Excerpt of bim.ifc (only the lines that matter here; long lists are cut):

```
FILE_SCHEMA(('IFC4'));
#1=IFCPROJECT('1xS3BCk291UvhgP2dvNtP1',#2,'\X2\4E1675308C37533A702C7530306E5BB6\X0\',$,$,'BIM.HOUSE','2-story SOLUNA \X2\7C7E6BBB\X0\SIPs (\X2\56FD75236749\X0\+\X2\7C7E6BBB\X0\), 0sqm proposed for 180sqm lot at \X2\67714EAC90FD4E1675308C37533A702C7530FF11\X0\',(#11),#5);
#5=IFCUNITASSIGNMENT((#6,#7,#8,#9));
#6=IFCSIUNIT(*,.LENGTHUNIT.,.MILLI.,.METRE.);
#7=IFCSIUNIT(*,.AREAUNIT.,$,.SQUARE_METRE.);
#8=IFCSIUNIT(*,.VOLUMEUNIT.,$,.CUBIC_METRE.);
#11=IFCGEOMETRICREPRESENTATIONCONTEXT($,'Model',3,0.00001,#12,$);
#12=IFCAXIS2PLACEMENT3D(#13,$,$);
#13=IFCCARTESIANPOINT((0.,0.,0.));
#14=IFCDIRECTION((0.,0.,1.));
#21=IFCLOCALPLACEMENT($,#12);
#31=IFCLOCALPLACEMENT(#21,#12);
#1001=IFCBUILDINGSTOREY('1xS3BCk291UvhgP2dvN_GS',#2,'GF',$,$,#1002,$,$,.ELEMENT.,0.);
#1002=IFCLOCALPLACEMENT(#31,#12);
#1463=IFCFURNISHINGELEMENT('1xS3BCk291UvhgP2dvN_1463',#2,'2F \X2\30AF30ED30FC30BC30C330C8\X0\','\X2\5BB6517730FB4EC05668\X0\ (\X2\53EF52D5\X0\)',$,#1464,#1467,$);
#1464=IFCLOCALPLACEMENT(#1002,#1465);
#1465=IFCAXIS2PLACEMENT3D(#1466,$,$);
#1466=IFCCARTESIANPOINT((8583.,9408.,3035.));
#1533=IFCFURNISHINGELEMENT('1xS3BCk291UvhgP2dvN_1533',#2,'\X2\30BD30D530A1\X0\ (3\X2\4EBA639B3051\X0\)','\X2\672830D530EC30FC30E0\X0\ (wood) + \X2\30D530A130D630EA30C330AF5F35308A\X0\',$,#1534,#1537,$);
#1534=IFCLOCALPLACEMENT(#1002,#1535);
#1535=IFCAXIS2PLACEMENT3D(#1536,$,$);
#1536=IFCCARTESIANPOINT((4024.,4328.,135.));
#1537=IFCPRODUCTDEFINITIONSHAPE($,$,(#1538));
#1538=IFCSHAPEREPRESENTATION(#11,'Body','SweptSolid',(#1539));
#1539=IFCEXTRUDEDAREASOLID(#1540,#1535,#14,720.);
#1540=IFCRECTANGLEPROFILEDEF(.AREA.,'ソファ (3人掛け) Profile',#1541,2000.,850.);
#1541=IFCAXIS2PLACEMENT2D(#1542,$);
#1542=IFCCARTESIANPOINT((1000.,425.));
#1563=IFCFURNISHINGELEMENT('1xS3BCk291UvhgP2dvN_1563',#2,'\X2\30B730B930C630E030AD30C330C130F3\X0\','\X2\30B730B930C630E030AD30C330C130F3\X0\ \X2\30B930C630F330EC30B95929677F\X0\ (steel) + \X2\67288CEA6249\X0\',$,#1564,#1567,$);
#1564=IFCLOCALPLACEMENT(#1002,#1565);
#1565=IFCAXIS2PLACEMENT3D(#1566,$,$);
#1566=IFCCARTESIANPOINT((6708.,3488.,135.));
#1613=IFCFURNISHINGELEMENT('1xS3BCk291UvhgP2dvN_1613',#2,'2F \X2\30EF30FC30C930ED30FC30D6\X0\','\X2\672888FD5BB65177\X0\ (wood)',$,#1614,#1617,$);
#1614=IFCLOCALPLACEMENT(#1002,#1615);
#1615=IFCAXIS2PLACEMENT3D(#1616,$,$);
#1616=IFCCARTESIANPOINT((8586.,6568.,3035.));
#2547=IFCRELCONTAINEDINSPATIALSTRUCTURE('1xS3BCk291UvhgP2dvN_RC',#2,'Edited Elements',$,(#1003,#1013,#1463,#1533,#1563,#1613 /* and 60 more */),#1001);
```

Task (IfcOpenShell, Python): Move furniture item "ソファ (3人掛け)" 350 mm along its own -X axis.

```python
import ifcopenshell
import ifcopenshell.api.geometry
import ifcopenshell.util.placement
import ifcopenshell.util.unit

model = ifcopenshell.open("bim.ifc")
unit_scale = ifcopenshell.util.unit.calculate_unit_scale(model)

item = model.by_id(1533)
matrix = ifcopenshell.util.placement.get_local_placement(item.ObjectPlacement)
matrix[:3, 3] -= matrix[:3, 0] * 0.35 / unit_scale
ifcopenshell.api.geometry.edit_object_placement(model, product=item, matrix=matrix, is_si=False)

print(ifcopenshell.util.placement.get_local_placement(item.ObjectPlacement).round(3) + 0.0)

model.write("bim_edited.ifc")
```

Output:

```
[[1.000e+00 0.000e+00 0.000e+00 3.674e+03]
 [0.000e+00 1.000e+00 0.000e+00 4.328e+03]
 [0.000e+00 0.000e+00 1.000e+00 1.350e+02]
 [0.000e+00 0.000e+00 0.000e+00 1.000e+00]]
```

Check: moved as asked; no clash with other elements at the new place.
